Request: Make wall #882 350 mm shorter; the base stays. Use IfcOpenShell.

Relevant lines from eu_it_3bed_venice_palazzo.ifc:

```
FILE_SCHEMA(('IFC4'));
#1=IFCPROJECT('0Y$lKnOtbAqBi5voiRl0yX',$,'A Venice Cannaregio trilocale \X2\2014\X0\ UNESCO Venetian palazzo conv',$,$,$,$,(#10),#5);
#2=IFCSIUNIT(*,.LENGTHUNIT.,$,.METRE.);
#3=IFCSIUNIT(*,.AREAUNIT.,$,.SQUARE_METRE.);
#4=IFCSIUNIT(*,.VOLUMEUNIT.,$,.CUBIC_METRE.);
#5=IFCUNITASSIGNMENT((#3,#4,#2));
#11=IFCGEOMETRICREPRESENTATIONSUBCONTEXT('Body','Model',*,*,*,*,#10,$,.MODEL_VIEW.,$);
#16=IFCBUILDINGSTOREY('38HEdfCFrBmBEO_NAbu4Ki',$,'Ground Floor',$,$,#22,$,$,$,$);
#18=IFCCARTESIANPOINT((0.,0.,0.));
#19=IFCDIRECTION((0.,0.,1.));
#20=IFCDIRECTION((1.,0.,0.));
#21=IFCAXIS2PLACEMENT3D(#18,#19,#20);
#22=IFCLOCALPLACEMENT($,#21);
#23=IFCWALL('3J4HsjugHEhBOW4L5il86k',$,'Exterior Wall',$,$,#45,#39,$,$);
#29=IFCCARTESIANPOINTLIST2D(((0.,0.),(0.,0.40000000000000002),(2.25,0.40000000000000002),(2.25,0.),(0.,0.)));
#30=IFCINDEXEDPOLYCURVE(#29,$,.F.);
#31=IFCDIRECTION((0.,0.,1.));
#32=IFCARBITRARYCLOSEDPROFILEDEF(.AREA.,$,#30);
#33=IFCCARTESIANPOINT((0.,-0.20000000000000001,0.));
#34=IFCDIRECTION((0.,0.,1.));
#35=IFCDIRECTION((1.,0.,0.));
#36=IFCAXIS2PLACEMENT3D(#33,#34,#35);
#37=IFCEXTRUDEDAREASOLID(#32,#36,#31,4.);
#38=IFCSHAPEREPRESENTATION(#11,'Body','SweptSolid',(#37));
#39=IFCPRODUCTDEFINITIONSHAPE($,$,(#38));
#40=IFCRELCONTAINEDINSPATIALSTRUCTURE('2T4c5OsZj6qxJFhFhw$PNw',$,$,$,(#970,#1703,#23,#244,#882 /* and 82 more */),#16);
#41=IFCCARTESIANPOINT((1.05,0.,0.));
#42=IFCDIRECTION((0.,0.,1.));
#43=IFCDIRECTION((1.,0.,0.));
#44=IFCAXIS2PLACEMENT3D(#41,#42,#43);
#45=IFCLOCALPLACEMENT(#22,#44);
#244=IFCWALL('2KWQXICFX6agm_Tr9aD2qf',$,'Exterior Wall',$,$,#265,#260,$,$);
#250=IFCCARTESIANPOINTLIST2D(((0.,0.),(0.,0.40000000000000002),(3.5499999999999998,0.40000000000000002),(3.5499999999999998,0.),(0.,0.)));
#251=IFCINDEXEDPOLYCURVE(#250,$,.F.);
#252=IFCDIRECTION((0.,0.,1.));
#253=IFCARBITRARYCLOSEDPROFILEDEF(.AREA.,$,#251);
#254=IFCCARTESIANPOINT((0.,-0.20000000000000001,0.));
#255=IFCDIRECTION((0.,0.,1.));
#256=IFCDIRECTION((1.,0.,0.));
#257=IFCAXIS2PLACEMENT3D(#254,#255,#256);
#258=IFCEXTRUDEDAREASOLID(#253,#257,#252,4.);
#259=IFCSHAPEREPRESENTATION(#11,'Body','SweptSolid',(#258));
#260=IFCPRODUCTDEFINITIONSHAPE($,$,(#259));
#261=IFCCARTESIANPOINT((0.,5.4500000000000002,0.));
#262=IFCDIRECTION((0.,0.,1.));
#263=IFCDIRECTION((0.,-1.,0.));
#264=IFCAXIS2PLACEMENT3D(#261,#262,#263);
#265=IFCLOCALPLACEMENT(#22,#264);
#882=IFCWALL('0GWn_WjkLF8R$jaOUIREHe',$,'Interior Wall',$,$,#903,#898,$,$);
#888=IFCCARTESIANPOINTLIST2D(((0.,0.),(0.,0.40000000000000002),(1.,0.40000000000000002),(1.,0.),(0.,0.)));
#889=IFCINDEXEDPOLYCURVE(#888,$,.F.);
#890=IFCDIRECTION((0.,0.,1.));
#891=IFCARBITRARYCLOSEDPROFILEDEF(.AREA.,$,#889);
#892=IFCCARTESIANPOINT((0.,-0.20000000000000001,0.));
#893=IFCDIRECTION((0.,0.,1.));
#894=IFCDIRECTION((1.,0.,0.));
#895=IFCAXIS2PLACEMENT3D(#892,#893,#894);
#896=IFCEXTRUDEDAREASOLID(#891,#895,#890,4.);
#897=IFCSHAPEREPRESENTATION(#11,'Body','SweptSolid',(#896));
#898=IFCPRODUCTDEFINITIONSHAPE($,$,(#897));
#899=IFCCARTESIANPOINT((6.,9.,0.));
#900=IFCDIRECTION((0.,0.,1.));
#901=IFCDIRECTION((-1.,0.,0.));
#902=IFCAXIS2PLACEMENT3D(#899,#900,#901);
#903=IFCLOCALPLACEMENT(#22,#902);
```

```python
import ifcopenshell
import ifcopenshell.geom
import ifcopenshell.util.representation
import ifcopenshell.util.shape
import ifcopenshell.util.unit

model = ifcopenshell.open("eu_it_3bed_venice_palazzo.ifc")
unit_scale = ifcopenshell.util.unit.calculate_unit_scale(model)
settings = ifcopenshell.geom.settings()


def volume(element):
    """Net volume in cubic metres, openings subtracted."""
    shape = ifcopenshell.geom.create_shape(settings, element)
    return ifcopenshell.util.shape.get_volume(shape.geometry)


wall = model.by_id(882)
before = volume(wall)

body = ifcopenshell.util.representation.get_representation(wall, "Model", "Body")
solid = body.Items[0]
old_height = solid.Depth
solid.Depth -= 0.35 / unit_scale
after = volume(wall)

print(f"height {old_height:g} -> {solid.Depth:g}, volume {before:.3f} -> {after:.3f} m3")

model.write("eu_it_3bed_venice_palazzo_v2.ifc")
```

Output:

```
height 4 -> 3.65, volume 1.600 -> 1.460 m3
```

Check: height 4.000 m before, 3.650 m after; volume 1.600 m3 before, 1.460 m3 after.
